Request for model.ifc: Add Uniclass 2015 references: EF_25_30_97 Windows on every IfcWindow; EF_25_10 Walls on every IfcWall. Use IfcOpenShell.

First a look at what the model holds.

```python
import ifcopenshell

model = ifcopenshell.open("model.ifc")
print(model.schema)
print("classifications:", [c.Name for c in model.by_type("IfcClassification")])
for ifc_class in ("IfcDoor", "IfcRoof", "IfcStair", "IfcWall", "IfcWindow"):
    print(ifc_class, len(model.by_type(ifc_class)))
```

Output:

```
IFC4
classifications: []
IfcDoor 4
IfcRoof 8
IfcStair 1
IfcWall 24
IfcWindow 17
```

```python
import ifcopenshell
import ifcopenshell.api.classification

model = ifcopenshell.open("model.ifc")

system = ifcopenshell.api.classification.add_classification(model, classification="Uniclass 2015")

codes = {
    "IfcWindow": ("EF_25_30_97", "Windows"),
    "IfcWall": ("EF_25_10", "Walls"),
}
for ifc_class, (code, name) in codes.items():
    products = model.by_type(ifc_class)
    ifcopenshell.api.classification.add_reference(
        model, products=products, classification=system, identification=code, name=name
    )
    print(code, len(products))

model.write("model_v2.ifc")
```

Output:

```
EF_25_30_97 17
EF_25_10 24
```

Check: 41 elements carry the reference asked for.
